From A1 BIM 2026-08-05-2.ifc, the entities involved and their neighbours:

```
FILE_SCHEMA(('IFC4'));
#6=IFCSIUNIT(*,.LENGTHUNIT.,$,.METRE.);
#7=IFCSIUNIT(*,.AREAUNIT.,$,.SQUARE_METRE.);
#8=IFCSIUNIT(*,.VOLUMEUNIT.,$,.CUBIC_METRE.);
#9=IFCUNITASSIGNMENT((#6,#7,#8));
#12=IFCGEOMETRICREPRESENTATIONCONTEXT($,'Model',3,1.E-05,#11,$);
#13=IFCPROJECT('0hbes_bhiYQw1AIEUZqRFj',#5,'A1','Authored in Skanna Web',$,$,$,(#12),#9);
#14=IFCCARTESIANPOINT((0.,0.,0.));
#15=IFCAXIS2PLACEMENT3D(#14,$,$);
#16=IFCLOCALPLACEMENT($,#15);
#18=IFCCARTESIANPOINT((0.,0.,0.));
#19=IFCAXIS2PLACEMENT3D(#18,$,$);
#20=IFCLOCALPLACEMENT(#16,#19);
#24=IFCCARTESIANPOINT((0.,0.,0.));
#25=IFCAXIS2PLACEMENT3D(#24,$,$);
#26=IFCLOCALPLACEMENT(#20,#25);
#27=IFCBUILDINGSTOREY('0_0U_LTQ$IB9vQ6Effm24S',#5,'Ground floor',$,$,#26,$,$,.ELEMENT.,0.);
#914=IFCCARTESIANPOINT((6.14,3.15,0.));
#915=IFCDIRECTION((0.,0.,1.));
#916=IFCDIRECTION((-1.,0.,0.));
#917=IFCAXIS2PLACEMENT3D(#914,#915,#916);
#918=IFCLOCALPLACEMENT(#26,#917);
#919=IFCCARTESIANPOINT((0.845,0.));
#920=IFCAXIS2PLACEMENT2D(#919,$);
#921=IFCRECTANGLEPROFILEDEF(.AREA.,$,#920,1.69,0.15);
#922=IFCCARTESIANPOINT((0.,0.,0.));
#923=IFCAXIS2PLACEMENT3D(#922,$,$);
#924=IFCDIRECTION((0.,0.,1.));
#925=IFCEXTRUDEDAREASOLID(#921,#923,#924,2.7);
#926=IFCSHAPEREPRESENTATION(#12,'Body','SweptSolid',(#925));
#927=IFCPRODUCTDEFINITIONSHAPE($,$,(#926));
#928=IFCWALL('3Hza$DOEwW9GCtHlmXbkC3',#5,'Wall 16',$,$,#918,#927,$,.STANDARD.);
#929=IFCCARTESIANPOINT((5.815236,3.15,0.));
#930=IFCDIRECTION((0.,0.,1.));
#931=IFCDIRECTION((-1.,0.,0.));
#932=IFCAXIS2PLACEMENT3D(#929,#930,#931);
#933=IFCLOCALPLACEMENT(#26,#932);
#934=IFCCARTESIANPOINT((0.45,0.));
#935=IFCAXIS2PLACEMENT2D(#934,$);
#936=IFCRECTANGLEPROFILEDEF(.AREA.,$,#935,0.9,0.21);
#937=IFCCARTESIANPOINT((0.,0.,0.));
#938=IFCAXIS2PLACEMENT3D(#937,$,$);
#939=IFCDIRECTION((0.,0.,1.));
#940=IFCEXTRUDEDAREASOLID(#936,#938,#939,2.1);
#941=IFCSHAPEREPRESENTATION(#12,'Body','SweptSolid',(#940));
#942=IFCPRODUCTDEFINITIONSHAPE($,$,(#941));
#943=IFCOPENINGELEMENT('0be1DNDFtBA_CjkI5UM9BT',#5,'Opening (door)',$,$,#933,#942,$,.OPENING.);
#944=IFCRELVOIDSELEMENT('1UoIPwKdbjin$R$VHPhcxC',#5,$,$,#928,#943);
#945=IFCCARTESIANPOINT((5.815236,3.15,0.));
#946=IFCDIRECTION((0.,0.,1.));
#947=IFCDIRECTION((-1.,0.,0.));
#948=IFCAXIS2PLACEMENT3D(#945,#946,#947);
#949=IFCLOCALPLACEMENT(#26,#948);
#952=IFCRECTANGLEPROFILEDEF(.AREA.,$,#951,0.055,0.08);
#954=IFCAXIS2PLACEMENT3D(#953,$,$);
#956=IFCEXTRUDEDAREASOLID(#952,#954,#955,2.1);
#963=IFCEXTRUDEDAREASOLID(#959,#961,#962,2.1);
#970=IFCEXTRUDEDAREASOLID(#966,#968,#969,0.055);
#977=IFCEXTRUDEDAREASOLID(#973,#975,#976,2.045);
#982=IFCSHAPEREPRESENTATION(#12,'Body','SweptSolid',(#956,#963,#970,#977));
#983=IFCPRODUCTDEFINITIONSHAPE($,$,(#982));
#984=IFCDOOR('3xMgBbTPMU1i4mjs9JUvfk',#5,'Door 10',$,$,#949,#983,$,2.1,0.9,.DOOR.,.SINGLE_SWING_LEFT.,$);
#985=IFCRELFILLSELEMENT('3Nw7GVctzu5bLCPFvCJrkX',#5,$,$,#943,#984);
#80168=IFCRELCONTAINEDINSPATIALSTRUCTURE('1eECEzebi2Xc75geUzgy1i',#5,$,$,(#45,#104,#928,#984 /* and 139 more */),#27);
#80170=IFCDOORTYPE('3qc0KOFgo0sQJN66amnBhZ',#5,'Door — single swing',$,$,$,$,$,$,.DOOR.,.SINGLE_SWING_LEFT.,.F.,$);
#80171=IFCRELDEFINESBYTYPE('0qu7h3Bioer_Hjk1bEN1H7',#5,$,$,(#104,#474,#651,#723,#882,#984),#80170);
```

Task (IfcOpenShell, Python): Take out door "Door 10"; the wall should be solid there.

```python
import ifcopenshell
import ifcopenshell.api.feature
import ifcopenshell.api.root
import ifcopenshell.geom
import ifcopenshell.util.shape

model = ifcopenshell.open("A1 BIM 2026-08-05-2.ifc")
settings = ifcopenshell.geom.settings()


def volume(element):
    """Net volume in cubic metres, openings subtracted."""
    shape = ifcopenshell.geom.create_shape(settings, element)
    return ifcopenshell.util.shape.get_volume(shape.geometry)


door = model.by_id(984)
opening = door.FillsVoids[0].RelatingOpeningElement
wall = opening.VoidsElements[0].RelatingBuildingElement
before = volume(wall)

ifcopenshell.api.root.remove_product(model, product=door)
ifcopenshell.api.feature.remove_feature(model, feature=opening)

after = volume(wall)

print(f"wall volume {before:.3f} -> {after:.3f} m3")

model.write("A1 BIM 2026-08-05-2_rev.ifc")
```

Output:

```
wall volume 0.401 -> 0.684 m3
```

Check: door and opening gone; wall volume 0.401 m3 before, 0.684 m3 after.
